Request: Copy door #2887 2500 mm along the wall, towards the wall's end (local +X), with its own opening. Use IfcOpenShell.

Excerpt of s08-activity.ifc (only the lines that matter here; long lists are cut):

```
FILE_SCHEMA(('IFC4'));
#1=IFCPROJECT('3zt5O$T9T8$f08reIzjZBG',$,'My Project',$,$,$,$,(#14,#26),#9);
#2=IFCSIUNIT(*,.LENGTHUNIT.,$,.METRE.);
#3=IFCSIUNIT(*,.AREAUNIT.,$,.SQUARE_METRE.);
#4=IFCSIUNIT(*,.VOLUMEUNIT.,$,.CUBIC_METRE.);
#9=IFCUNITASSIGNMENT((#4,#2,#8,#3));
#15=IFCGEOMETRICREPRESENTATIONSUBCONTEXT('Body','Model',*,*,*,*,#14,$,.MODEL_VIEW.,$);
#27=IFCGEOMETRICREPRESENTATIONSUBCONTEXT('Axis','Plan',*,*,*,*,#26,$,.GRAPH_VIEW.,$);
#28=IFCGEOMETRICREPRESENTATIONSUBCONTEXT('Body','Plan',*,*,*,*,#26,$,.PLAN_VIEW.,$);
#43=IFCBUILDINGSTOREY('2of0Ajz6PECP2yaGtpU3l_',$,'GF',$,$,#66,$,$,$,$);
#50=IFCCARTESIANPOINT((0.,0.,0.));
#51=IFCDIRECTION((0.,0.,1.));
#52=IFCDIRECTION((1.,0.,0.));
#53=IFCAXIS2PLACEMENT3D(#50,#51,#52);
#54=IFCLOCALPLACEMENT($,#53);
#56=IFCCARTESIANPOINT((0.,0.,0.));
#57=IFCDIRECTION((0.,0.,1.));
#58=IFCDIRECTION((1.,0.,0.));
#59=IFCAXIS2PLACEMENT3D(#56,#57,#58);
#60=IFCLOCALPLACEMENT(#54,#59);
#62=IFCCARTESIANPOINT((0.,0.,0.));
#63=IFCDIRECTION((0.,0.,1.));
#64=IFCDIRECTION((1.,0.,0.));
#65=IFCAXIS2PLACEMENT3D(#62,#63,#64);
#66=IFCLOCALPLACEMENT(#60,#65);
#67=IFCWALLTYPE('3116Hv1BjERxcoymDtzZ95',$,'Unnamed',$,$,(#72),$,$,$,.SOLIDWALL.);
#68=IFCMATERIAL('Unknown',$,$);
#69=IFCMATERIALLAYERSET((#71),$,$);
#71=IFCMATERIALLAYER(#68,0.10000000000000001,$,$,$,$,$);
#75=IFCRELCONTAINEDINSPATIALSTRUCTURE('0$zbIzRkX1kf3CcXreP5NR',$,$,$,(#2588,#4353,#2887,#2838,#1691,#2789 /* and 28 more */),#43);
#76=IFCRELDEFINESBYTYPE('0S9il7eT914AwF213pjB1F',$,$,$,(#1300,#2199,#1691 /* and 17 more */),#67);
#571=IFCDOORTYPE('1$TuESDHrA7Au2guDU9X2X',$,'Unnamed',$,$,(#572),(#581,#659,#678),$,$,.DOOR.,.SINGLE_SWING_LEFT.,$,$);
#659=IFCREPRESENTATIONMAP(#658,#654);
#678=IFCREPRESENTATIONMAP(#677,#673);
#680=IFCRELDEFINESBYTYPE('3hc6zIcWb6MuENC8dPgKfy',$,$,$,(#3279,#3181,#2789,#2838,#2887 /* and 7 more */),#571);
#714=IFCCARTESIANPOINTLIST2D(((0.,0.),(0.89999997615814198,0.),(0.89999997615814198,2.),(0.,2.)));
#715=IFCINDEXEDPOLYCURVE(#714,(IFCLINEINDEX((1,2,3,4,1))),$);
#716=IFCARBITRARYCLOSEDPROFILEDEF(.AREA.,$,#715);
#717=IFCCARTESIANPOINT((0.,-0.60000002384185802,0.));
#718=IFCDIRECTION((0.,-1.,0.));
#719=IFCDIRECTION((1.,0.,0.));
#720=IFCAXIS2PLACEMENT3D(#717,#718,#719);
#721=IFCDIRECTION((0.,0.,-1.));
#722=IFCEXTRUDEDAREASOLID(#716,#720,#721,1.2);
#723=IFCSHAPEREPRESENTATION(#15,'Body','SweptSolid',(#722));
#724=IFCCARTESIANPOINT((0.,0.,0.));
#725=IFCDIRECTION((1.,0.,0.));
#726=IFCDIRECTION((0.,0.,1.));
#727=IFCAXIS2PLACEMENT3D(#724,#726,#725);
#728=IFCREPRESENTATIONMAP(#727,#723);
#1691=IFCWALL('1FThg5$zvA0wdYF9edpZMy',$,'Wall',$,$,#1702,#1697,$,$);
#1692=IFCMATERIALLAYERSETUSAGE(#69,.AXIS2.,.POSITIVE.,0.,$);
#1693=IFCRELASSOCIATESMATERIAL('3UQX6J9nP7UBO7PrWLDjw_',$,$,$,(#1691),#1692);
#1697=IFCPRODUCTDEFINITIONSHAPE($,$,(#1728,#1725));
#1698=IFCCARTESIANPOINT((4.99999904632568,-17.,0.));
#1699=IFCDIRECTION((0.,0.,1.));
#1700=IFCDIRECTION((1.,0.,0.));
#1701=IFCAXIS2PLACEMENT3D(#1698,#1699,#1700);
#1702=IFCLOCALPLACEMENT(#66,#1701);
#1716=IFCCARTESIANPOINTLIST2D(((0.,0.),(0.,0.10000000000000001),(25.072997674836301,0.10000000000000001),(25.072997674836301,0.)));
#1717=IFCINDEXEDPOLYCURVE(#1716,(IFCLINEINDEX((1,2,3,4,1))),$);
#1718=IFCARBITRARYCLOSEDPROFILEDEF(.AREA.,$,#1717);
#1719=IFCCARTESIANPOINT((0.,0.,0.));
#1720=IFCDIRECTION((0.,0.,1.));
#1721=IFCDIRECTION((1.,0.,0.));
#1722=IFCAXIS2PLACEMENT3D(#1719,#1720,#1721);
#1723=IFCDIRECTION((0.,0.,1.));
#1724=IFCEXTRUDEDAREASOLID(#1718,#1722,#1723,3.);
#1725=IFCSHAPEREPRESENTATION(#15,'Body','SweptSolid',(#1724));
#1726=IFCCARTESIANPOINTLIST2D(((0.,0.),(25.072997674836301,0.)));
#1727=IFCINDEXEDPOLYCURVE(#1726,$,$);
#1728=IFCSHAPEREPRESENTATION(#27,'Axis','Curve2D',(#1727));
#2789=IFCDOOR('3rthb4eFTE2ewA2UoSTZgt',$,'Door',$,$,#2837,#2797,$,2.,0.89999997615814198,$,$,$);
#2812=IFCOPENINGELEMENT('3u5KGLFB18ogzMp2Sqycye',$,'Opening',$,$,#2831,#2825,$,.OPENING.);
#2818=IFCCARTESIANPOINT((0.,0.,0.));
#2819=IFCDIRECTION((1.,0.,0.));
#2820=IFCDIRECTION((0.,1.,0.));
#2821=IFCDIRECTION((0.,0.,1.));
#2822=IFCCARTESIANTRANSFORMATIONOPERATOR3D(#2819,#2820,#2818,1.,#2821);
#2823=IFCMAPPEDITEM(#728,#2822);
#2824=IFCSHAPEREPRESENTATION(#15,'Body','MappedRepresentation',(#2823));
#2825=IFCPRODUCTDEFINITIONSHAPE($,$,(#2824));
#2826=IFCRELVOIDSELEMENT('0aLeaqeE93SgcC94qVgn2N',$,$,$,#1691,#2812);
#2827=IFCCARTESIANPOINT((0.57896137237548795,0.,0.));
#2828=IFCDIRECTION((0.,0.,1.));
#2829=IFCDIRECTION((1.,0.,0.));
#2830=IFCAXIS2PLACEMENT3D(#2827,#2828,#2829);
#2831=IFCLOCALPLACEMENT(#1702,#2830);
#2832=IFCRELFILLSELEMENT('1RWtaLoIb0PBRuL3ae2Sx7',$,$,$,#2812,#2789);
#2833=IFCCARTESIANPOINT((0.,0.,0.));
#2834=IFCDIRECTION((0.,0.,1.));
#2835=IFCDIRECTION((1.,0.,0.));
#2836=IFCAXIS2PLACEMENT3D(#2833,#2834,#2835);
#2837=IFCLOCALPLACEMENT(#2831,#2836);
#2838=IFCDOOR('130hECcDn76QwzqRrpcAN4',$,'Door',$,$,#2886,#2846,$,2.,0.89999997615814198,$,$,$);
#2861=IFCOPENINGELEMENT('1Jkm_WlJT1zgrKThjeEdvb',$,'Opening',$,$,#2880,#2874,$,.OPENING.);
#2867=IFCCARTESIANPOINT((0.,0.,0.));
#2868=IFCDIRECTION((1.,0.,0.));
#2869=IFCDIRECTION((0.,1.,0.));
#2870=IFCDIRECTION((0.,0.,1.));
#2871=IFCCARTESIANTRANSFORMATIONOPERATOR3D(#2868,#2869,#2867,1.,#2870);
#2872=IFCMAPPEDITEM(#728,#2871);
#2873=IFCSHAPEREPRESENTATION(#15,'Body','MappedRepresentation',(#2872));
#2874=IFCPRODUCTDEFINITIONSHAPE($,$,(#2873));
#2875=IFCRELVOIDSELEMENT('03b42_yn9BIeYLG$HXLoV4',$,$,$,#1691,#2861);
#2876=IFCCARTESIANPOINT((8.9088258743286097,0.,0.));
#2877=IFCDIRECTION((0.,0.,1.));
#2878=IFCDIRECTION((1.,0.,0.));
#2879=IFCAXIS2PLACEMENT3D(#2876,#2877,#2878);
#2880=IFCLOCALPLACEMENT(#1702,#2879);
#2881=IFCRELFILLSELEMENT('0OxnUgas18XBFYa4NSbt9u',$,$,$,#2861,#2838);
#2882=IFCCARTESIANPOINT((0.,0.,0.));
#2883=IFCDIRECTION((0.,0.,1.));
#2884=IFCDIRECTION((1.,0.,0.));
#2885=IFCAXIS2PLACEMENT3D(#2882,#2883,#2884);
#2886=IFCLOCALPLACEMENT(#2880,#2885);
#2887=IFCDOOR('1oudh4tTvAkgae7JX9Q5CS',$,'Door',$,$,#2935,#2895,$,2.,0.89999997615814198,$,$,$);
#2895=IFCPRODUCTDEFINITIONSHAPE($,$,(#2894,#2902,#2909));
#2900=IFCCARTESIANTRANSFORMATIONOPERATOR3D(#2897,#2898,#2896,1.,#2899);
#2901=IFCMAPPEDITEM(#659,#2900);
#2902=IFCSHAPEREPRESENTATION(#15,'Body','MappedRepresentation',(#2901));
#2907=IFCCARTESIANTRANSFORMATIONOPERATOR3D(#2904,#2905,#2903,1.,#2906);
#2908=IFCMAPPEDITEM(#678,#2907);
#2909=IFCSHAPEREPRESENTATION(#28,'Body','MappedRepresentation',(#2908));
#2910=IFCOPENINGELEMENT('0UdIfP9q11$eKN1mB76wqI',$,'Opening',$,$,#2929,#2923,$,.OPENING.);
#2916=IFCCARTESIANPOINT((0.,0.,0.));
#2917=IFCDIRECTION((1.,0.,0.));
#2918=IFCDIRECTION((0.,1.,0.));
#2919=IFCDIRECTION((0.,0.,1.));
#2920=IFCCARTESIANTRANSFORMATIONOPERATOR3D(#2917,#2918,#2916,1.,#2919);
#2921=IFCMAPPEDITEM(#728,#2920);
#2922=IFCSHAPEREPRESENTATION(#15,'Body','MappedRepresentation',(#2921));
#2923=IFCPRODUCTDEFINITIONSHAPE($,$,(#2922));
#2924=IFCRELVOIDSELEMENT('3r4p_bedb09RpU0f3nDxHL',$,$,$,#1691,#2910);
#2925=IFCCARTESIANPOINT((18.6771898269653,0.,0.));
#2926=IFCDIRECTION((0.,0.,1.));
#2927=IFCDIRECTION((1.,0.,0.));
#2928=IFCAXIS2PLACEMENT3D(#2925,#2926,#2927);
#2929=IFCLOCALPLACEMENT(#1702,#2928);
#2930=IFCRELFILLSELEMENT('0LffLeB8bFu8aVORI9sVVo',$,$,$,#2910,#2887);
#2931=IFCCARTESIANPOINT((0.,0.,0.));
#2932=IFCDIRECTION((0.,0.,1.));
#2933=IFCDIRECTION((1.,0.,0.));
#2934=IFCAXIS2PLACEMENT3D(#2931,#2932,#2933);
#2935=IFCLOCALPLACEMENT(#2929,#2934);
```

```python
import ifcopenshell
import ifcopenshell.api.feature
import ifcopenshell.api.geometry
import ifcopenshell.api.root
import ifcopenshell.geom
import ifcopenshell.util.element
import ifcopenshell.util.placement
import ifcopenshell.util.shape

model = ifcopenshell.open("s08-activity.ifc")
settings = ifcopenshell.geom.settings()


def volume(element):
    """Net volume in cubic metres, openings subtracted."""
    shape = ifcopenshell.geom.create_shape(settings, element)
    return ifcopenshell.util.shape.get_volume(shape.geometry)


door = model.by_guid("1oudh4tTvAkgae7JX9Q5CS")
opening = door.FillsVoids[0].RelatingOpeningElement
wall = opening.VoidsElements[0].RelatingBuildingElement
before = volume(wall)
shift = ifcopenshell.util.placement.get_local_placement(wall.ObjectPlacement)[:3, 0] * 2.5

# copy_class copies the void relationship, type, container and properties, but no geometry.
new_opening = ifcopenshell.api.root.copy_class(model, product=opening)
new_opening.Representation = ifcopenshell.util.element.copy_deep(
    model, opening.Representation, exclude=["IfcGeometricRepresentationContext", "IfcRepresentationMap"]
)
new_door = ifcopenshell.api.root.copy_class(model, product=door)
new_door.Representation = ifcopenshell.util.element.copy_deep(
    model, door.Representation, exclude=["IfcGeometricRepresentationContext", "IfcRepresentationMap"]
)
ifcopenshell.api.feature.add_filling(model, opening=new_opening, element=new_door)

for old, new in ((opening, new_opening), (door, new_door)):
    matrix = ifcopenshell.util.placement.get_local_placement(old.ObjectPlacement)
    matrix[:3, 3] += shift
    ifcopenshell.api.geometry.edit_object_placement(model, product=new, matrix=matrix, is_si=False)

after = volume(wall)

print(f"wall volume {before:.3f} -> {after:.3f} m3")

model.write("s08-activity-out.ifc")
```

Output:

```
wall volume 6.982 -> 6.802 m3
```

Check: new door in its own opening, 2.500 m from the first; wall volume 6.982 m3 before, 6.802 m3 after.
